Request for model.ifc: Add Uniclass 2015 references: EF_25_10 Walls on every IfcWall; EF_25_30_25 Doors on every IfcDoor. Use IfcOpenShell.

First a look at what the model holds.

```python
import ifcopenshell

model = ifcopenshell.open("model.ifc")
print(model.schema)
print("classifications:", [c.Name for c in model.by_type("IfcClassification")])
for ifc_class in ("IfcDoor", "IfcRoof", "IfcStair", "IfcWall", "IfcWindow"):
    print(ifc_class, len(model.by_type(ifc_class)))
```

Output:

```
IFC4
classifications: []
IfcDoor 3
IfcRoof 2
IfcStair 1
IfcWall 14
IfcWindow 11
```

```python
import ifcopenshell
import ifcopenshell.api.classification

model = ifcopenshell.open("model.ifc")

system = ifcopenshell.api.classification.add_classification(model, classification="Uniclass 2015")

codes = {
    "IfcWall": ("EF_25_10", "Walls"),
    "IfcDoor": ("EF_25_30_25", "Doors"),
}
for ifc_class, (code, name) in codes.items():
    products = model.by_type(ifc_class)
    ifcopenshell.api.classification.add_reference(
        model, products=products, classification=system, identification=code, name=name
    )
    print(code, len(products))

model.write("model_updated.ifc")
```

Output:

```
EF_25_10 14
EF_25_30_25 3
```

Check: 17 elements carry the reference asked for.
